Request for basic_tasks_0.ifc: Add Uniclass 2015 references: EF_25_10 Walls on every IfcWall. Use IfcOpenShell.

First a look at what the model holds.

```python
import ifcopenshell

model = ifcopenshell.open("basic_tasks_0.ifc")
print(model.schema)
print("classifications:", [c.Name for c in model.by_type("IfcClassification")])
for ifc_class in ("IfcDoor", "IfcRoof", "IfcStair", "IfcWall", "IfcWindow"):
    print(ifc_class, len(model.by_type(ifc_class)))
```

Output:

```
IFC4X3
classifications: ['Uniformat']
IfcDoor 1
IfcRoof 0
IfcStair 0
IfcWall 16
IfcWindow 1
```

```python
import ifcopenshell
import ifcopenshell.api.classification

model = ifcopenshell.open("basic_tasks_0.ifc")

system = ifcopenshell.api.classification.add_classification(model, classification="Uniclass 2015")

codes = {
    "IfcWall": ("EF_25_10", "Walls"),
}
for ifc_class, (code, name) in codes.items():
    products = model.by_type(ifc_class)
    ifcopenshell.api.classification.add_reference(
        model, products=products, classification=system, identification=code, name=name
    )
    print(code, len(products))

model.write("basic_tasks_0_edited.ifc")
```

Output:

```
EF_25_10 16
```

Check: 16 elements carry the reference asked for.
